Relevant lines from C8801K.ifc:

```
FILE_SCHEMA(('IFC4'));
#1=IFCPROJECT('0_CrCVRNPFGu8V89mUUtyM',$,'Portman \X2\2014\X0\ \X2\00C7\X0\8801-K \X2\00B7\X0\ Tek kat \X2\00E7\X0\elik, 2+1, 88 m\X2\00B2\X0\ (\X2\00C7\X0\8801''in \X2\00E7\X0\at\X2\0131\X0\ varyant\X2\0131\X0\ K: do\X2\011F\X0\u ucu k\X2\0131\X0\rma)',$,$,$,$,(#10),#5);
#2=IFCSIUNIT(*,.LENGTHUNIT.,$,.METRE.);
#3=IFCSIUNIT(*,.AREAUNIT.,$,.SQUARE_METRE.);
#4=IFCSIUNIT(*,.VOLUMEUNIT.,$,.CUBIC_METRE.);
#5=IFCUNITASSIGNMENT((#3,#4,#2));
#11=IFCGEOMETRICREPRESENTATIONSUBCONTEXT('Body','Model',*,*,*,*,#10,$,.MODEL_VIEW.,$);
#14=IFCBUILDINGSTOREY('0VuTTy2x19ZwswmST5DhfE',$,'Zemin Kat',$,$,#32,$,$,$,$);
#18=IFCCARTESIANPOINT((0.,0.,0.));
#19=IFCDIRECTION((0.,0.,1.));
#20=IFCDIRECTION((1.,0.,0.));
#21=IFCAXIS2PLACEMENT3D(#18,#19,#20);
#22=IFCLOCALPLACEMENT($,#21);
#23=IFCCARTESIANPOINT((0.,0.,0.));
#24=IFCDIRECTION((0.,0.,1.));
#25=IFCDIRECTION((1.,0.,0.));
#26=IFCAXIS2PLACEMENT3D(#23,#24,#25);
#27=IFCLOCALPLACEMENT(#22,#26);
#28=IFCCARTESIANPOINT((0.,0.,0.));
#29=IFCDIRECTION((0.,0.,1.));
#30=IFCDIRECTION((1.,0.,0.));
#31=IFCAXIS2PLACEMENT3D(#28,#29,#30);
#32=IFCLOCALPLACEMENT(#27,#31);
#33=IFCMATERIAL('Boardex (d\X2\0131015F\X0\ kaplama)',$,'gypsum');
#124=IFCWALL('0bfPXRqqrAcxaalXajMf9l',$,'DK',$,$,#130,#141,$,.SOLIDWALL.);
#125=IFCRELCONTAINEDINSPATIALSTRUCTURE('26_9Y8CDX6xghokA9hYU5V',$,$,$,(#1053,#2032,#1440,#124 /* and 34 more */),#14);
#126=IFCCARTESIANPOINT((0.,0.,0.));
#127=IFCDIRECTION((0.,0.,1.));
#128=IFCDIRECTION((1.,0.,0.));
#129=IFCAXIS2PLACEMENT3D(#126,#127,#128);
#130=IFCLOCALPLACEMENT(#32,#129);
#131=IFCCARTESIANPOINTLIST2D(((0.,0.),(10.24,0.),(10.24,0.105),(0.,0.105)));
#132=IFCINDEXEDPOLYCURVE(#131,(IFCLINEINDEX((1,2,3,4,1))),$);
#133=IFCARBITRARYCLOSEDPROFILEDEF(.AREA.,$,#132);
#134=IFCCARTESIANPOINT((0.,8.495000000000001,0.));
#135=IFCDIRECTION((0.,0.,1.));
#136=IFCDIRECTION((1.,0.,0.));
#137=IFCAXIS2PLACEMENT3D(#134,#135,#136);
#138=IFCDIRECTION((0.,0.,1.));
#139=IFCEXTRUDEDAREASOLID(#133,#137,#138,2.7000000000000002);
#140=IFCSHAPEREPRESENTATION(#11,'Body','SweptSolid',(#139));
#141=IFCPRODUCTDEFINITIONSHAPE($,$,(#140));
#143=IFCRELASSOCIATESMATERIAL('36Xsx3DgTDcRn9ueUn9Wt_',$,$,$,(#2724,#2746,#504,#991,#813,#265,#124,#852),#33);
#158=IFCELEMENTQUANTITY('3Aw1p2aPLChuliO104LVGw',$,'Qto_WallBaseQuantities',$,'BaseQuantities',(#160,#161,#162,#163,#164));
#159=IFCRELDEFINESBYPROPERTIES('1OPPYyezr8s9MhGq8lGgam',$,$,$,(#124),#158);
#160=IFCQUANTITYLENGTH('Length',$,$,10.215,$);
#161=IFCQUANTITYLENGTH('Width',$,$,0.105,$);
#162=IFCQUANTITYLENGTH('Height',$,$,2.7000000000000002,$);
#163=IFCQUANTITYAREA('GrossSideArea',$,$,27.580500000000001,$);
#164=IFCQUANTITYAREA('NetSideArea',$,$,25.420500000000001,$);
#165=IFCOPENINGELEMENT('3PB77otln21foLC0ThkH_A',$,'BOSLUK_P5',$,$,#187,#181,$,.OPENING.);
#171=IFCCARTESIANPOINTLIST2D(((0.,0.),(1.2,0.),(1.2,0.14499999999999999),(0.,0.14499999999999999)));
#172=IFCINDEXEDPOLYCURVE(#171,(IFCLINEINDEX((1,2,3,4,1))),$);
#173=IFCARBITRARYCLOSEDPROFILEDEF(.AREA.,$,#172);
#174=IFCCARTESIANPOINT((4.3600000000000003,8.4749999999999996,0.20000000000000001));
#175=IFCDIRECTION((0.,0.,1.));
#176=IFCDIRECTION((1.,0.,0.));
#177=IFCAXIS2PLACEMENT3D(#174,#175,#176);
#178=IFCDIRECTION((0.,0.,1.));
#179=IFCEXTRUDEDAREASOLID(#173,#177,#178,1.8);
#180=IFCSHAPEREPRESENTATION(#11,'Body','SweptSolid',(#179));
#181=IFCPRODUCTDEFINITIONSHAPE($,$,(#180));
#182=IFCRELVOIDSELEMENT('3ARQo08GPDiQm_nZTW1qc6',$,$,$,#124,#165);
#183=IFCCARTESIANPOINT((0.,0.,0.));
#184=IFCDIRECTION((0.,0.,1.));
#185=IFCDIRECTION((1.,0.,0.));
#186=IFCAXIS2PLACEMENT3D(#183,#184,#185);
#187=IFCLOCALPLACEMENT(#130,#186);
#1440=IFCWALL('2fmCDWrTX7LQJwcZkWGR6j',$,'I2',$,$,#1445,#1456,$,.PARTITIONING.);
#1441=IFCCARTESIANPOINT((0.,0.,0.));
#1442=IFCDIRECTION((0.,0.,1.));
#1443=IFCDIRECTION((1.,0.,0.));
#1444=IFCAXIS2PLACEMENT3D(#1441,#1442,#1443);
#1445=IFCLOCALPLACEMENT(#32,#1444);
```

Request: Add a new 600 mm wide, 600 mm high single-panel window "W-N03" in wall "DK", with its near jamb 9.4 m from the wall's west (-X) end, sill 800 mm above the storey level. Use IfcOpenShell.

```python
import numpy as np
import ifcopenshell
import ifcopenshell.api.feature
import ifcopenshell.api.geometry
import ifcopenshell.api.pset
import ifcopenshell.api.root
import ifcopenshell.api.spatial
import ifcopenshell.geom
import ifcopenshell.util.element
import ifcopenshell.util.placement
import ifcopenshell.util.representation
import ifcopenshell.util.shape
import ifcopenshell.util.unit

model = ifcopenshell.open("C8801K.ifc")
unit_scale = ifcopenshell.util.unit.calculate_unit_scale(model)
area_scale = ifcopenshell.util.unit.calculate_unit_scale(model, "AREAUNIT")
settings = ifcopenshell.geom.settings()


def volume(element):
    """Net volume in cubic metres, openings subtracted."""
    shape = ifcopenshell.geom.create_shape(settings, element)
    return ifcopenshell.util.shape.get_volume(shape.geometry)


wall = model.by_guid("0bfPXRqqrAcxaalXajMf9l")
storey = ifcopenshell.util.element.get_container(wall, ifc_class="IfcBuildingStorey")
context = ifcopenshell.util.representation.get_context(model, "Model", "Body", "MODEL_VIEW")
before = volume(wall)

width, height, from_end, sill = 0.6, 0.6, 9.4, 0.8  # metres

# The wall runs along its own X axis, and the end named is its -X end.
wall_shape = ifcopenshell.geom.create_shape(settings, wall)
x, y, z = ifcopenshell.util.shape.get_vertices(wall_shape.geometry).T
start = x.min() + from_end
face, thickness = float(y.min()), float(y.max() - y.min())
wall_matrix = ifcopenshell.util.placement.get_local_placement(wall.ObjectPlacement)
level = ifcopenshell.util.placement.get_local_placement(storey.ObjectPlacement)[2, 3]


def in_wall(x, y):
    """Placement at x, y metres in the wall's axes, at sill height."""
    matrix = wall_matrix.copy()
    matrix[:, 3] = wall_matrix @ np.array([x / unit_scale, y / unit_scale, 0.0, 1.0])
    matrix[2, 3] = level + sill / unit_scale
    return matrix


# Opening: a box that overshoots both wall faces by 50 mm.
opening = ifcopenshell.api.root.create_entity(model, ifc_class="IfcOpeningElement", predefined_type="OPENING")
box = ifcopenshell.api.geometry.add_wall_representation(
    model, context=context, length=width, height=height, thickness=thickness + 0.1
)
ifcopenshell.api.geometry.assign_representation(model, product=opening, representation=box)
ifcopenshell.api.geometry.edit_object_placement(model, product=opening, matrix=in_wall(start, face - 0.05), is_si=False)
ifcopenshell.api.feature.add_feature(model, feature=opening, element=wall)

window = ifcopenshell.api.root.create_entity(model, ifc_class="IfcWindow", name="W-N03", predefined_type="WINDOW")
window.OverallWidth, window.OverallHeight = width / unit_scale, height / unit_scale
window.PartitioningType = "SINGLE_PANEL"
body = ifcopenshell.api.geometry.add_window_representation(
    model,
    context=context,
    overall_width=window.OverallWidth,
    overall_height=window.OverallHeight,
    partition_type="SINGLE_PANEL",
)
ifcopenshell.api.geometry.assign_representation(model, product=window, representation=body)
ifcopenshell.api.spatial.assign_container(model, products=[window], relating_structure=storey)
ifcopenshell.api.feature.add_filling(model, opening=opening, element=window)

# Centre the window in the wall's thickness.
ifcopenshell.api.geometry.edit_object_placement(model, product=window, matrix=in_wall(start, face), is_si=False)
window_shape = ifcopenshell.geom.create_shape(settings, window)
depth = ifcopenshell.util.shape.get_vertices(window_shape.geometry)[:, 1]
offset = face + thickness / 2 - (depth.min() + depth.max()) / 2
ifcopenshell.api.geometry.edit_object_placement(model, product=window, matrix=in_wall(start, offset), is_si=False)

after = volume(wall)

# Update the wall's stored quantities.
qto = model.by_id(ifcopenshell.util.element.get_pset(wall, "Qto_WallBaseQuantities", should_inherit=False)["id"])
ifcopenshell.api.pset.edit_qto(model, qto=qto, properties={"NetSideArea": after / thickness / area_scale})

print(f"wall volume {before:.3f} -> {after:.3f} m3")

model.write("C8801K-out.ifc")
```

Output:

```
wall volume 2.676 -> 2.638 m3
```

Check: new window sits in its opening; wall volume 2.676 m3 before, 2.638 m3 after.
